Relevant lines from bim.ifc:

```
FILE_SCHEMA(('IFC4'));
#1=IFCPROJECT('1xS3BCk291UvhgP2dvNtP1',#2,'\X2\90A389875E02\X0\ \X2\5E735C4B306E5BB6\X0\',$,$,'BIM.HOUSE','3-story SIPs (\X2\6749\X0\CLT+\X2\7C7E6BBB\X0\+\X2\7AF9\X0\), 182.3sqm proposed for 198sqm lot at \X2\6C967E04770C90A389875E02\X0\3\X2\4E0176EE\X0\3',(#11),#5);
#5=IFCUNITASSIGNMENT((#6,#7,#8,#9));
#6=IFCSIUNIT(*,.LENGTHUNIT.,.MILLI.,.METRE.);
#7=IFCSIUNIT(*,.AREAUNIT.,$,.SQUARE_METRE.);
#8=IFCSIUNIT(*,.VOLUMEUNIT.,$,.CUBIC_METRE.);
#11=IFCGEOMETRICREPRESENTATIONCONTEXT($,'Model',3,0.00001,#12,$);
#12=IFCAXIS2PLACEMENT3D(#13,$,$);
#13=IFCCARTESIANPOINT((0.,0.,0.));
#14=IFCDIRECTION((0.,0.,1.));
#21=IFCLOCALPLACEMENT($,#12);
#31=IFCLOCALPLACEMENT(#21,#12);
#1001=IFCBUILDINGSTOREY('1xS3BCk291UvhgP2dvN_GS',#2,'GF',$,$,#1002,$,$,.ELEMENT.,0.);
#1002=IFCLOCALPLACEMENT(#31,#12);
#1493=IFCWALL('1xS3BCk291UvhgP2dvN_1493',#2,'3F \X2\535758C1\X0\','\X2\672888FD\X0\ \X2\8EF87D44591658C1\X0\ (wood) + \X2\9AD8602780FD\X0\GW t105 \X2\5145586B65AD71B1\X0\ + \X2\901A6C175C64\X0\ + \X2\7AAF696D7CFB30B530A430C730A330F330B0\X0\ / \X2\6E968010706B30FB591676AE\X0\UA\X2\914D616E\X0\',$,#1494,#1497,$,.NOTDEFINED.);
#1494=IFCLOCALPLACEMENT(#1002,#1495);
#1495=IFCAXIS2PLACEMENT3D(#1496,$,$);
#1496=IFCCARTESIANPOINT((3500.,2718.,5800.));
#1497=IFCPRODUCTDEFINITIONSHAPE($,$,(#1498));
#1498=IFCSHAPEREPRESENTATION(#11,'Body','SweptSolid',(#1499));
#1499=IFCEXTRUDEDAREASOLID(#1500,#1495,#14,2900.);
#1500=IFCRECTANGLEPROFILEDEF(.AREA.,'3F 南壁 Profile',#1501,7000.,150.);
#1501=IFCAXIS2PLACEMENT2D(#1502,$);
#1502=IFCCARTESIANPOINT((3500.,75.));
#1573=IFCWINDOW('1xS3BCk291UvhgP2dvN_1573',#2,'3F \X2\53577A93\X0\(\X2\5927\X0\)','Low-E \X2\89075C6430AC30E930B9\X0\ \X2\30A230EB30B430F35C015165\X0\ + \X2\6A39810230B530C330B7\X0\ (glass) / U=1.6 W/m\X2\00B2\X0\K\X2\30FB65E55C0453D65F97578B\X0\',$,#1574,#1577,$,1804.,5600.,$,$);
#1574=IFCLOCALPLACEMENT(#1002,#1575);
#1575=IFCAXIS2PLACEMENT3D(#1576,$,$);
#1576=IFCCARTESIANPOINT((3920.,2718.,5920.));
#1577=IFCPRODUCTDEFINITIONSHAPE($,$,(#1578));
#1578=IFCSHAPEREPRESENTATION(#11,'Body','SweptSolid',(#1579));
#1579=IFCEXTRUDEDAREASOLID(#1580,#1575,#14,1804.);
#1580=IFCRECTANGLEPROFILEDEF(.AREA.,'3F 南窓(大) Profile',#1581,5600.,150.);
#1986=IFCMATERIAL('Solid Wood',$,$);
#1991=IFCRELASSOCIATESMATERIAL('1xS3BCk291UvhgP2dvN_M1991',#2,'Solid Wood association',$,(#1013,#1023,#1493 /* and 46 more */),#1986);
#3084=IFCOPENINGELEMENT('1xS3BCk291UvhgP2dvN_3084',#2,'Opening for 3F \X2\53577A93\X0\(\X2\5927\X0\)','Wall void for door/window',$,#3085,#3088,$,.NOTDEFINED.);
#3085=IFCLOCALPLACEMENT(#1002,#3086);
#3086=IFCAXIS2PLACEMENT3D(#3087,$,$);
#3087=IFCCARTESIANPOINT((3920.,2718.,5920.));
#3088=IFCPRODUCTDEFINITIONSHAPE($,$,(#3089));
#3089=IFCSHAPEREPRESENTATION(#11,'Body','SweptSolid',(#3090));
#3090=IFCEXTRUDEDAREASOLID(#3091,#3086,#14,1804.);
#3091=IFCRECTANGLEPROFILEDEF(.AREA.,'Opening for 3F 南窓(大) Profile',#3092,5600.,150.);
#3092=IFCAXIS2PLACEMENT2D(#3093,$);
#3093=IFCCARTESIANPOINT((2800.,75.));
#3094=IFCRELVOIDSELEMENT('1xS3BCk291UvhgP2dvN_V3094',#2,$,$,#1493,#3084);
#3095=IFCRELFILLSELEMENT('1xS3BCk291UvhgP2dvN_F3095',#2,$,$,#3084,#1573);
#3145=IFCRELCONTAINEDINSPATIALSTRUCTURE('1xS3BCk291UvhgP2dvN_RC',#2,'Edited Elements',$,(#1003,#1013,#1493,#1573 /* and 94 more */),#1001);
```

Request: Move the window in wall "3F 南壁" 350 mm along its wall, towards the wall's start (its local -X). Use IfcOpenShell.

```python
import ifcopenshell
import ifcopenshell.api.geometry
import ifcopenshell.util.placement

model = ifcopenshell.open("bim.ifc")

window = model.by_guid("1xS3BCk291UvhgP2dvN_1573")
opening = window.FillsVoids[0].RelatingOpeningElement
wall = opening.VoidsElements[0].RelatingBuildingElement

wall_matrix = ifcopenshell.util.placement.get_local_placement(wall.ObjectPlacement)
shift = wall_matrix[:3, 0] * -350.0
before = ifcopenshell.util.placement.get_local_placement(window.ObjectPlacement)[:3, 3].copy()

# The window is not placed relative to its opening, so move both.
for product in (opening, window):
    matrix = ifcopenshell.util.placement.get_local_placement(product.ObjectPlacement)
    matrix[:3, 3] += shift
    ifcopenshell.api.geometry.edit_object_placement(model, product=product, matrix=matrix, is_si=False)

after = ifcopenshell.util.placement.get_local_placement(window.ObjectPlacement)[:3, 3]
print("window moved by", (after - before).round(3) + 0.0)

model.write("bim-out.ifc")
```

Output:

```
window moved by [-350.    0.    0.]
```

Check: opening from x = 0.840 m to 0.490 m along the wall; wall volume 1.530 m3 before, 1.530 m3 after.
